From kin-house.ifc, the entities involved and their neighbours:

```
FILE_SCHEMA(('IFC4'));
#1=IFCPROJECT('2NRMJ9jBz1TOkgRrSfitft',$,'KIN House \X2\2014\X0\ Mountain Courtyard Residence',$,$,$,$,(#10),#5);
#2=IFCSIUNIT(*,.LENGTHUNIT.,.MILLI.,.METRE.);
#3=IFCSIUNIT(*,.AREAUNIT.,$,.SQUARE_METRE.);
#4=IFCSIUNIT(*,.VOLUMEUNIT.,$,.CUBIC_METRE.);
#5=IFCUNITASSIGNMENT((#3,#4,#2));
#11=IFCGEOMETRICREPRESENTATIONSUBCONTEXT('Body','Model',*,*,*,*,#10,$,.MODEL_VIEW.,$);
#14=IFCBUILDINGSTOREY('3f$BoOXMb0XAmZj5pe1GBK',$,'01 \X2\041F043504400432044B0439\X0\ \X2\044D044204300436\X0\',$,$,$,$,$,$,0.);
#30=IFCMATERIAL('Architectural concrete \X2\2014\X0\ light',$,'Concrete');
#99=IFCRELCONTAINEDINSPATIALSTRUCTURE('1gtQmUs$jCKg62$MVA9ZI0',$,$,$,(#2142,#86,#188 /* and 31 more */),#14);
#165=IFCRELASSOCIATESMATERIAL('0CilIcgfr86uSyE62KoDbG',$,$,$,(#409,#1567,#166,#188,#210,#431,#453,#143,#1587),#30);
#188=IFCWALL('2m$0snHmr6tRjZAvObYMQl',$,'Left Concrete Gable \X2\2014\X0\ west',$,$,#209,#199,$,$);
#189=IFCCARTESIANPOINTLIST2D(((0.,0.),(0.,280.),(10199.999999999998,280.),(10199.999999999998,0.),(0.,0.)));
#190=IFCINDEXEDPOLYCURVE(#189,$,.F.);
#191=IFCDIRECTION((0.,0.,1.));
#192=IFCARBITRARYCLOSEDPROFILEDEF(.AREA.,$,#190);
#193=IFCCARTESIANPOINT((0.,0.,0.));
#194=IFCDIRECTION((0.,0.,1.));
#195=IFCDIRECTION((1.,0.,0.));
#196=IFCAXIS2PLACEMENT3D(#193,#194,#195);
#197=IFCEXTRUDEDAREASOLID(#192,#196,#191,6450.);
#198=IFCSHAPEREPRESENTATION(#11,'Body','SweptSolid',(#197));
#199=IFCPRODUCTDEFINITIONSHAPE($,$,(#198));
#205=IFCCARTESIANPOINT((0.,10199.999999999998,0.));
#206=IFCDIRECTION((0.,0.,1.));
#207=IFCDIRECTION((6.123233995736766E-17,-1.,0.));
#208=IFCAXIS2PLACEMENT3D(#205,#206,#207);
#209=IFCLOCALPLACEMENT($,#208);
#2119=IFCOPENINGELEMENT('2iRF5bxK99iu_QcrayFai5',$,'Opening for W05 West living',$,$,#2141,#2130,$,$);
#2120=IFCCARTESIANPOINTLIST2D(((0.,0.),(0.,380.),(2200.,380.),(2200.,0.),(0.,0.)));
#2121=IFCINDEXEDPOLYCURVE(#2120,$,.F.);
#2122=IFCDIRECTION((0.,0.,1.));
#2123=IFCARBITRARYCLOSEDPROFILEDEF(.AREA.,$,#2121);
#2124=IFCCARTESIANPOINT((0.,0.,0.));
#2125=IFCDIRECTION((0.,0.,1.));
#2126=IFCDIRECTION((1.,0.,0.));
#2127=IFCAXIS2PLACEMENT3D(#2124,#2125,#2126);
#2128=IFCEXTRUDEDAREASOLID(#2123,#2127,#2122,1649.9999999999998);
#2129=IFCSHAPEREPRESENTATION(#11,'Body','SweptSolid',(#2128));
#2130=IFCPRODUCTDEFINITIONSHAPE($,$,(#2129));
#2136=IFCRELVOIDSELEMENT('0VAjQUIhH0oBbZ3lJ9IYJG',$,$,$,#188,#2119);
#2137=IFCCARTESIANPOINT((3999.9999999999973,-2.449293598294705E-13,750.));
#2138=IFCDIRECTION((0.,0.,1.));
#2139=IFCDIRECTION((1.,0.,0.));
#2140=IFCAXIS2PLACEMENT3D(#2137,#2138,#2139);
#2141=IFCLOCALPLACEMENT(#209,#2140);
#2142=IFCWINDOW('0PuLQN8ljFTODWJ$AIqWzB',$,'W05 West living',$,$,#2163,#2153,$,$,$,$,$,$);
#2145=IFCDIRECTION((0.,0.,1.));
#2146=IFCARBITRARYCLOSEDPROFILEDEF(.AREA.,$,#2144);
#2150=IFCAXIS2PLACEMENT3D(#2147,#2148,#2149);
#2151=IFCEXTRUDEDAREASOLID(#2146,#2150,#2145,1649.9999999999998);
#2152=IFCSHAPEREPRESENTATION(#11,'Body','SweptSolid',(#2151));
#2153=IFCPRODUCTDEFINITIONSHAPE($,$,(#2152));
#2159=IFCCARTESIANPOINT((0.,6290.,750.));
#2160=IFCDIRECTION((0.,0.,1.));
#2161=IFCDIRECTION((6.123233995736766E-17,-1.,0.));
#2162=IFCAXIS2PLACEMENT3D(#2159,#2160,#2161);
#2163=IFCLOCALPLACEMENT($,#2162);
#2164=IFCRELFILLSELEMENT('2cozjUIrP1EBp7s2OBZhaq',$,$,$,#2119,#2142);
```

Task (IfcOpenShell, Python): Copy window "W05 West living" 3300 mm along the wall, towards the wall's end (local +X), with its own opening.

```python
import ifcopenshell
import ifcopenshell.api.feature
import ifcopenshell.api.geometry
import ifcopenshell.api.root
import ifcopenshell.geom
import ifcopenshell.util.element
import ifcopenshell.util.placement
import ifcopenshell.util.shape

model = ifcopenshell.open("kin-house.ifc")
settings = ifcopenshell.geom.settings()


def volume(element):
    """Net volume in cubic metres, openings subtracted."""
    shape = ifcopenshell.geom.create_shape(settings, element)
    return ifcopenshell.util.shape.get_volume(shape.geometry)


window = model.by_id(2142)
opening = window.FillsVoids[0].RelatingOpeningElement
wall = opening.VoidsElements[0].RelatingBuildingElement
before = volume(wall)
shift = ifcopenshell.util.placement.get_local_placement(wall.ObjectPlacement)[:3, 0] * 3300.0

# copy_class copies the void relationship, type, container and properties, but no geometry.
new_opening = ifcopenshell.api.root.copy_class(model, product=opening)
new_opening.Representation = ifcopenshell.util.element.copy_deep(
    model, opening.Representation, exclude=["IfcGeometricRepresentationContext", "IfcRepresentationMap"]
)
new_window = ifcopenshell.api.root.copy_class(model, product=window)
new_window.Representation = ifcopenshell.util.element.copy_deep(
    model, window.Representation, exclude=["IfcGeometricRepresentationContext", "IfcRepresentationMap"]
)
ifcopenshell.api.feature.add_filling(model, opening=new_opening, element=new_window)

for old, new in ((opening, new_opening), (window, new_window)):
    matrix = ifcopenshell.util.placement.get_local_placement(old.ObjectPlacement)
    matrix[:3, 3] += shift
    ifcopenshell.api.geometry.edit_object_placement(model, product=new, matrix=matrix, is_si=False)

after = volume(wall)

print(f"wall volume {before:.3f} -> {after:.3f} m3")

model.write("kin-house_v2.ifc")
```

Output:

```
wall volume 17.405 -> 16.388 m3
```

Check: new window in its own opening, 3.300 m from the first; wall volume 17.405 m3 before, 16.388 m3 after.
